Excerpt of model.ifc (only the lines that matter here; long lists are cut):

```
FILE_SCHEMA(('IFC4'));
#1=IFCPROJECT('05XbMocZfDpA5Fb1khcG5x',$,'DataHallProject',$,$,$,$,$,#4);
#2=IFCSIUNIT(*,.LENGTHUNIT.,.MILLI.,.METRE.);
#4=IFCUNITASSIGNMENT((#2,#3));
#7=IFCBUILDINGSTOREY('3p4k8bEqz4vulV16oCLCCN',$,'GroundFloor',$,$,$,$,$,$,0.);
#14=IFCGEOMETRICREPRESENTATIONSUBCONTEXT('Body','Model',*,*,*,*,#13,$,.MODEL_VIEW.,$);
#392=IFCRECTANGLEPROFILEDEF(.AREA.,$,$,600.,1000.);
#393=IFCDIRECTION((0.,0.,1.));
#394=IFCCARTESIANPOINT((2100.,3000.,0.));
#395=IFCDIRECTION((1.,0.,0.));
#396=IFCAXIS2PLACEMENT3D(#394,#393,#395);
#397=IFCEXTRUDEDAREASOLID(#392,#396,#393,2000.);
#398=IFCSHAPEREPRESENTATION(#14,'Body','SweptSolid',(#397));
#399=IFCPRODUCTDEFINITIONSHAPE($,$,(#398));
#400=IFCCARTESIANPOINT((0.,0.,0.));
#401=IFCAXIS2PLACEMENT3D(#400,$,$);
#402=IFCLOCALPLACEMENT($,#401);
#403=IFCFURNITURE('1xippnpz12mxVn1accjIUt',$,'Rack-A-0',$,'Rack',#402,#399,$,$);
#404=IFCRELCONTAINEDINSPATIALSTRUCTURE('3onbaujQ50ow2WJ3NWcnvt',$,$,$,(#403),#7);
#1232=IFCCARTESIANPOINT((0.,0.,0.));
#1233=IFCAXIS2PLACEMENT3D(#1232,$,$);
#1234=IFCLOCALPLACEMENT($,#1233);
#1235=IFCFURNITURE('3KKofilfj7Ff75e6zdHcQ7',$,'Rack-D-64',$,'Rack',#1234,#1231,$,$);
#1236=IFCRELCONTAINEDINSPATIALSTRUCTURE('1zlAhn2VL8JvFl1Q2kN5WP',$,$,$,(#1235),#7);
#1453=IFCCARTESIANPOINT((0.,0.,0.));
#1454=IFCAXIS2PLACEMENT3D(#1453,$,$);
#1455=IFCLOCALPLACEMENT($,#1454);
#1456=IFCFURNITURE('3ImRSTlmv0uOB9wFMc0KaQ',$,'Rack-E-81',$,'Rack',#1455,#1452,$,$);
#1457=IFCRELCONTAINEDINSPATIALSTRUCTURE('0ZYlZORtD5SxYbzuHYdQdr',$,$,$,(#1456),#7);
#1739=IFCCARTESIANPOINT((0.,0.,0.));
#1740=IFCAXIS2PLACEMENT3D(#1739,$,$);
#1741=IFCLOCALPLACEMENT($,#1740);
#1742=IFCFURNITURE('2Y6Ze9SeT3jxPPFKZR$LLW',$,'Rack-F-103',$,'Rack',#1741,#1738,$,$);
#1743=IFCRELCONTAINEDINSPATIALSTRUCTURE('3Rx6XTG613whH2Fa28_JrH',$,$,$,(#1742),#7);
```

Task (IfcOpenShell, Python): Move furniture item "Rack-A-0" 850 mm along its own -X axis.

```python
import ifcopenshell
import ifcopenshell.api.geometry
import ifcopenshell.util.placement

model = ifcopenshell.open("model.ifc")

item = model.by_id(403)
matrix = ifcopenshell.util.placement.get_local_placement(item.ObjectPlacement)
matrix[:3, 3] -= matrix[:3, 0] * 850.0
ifcopenshell.api.geometry.edit_object_placement(model, product=item, matrix=matrix, is_si=False)

print(ifcopenshell.util.placement.get_local_placement(item.ObjectPlacement).round(3) + 0.0)

model.write("model_updated.ifc")
```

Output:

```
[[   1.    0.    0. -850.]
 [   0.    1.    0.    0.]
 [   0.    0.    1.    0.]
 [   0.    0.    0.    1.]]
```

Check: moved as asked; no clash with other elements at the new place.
